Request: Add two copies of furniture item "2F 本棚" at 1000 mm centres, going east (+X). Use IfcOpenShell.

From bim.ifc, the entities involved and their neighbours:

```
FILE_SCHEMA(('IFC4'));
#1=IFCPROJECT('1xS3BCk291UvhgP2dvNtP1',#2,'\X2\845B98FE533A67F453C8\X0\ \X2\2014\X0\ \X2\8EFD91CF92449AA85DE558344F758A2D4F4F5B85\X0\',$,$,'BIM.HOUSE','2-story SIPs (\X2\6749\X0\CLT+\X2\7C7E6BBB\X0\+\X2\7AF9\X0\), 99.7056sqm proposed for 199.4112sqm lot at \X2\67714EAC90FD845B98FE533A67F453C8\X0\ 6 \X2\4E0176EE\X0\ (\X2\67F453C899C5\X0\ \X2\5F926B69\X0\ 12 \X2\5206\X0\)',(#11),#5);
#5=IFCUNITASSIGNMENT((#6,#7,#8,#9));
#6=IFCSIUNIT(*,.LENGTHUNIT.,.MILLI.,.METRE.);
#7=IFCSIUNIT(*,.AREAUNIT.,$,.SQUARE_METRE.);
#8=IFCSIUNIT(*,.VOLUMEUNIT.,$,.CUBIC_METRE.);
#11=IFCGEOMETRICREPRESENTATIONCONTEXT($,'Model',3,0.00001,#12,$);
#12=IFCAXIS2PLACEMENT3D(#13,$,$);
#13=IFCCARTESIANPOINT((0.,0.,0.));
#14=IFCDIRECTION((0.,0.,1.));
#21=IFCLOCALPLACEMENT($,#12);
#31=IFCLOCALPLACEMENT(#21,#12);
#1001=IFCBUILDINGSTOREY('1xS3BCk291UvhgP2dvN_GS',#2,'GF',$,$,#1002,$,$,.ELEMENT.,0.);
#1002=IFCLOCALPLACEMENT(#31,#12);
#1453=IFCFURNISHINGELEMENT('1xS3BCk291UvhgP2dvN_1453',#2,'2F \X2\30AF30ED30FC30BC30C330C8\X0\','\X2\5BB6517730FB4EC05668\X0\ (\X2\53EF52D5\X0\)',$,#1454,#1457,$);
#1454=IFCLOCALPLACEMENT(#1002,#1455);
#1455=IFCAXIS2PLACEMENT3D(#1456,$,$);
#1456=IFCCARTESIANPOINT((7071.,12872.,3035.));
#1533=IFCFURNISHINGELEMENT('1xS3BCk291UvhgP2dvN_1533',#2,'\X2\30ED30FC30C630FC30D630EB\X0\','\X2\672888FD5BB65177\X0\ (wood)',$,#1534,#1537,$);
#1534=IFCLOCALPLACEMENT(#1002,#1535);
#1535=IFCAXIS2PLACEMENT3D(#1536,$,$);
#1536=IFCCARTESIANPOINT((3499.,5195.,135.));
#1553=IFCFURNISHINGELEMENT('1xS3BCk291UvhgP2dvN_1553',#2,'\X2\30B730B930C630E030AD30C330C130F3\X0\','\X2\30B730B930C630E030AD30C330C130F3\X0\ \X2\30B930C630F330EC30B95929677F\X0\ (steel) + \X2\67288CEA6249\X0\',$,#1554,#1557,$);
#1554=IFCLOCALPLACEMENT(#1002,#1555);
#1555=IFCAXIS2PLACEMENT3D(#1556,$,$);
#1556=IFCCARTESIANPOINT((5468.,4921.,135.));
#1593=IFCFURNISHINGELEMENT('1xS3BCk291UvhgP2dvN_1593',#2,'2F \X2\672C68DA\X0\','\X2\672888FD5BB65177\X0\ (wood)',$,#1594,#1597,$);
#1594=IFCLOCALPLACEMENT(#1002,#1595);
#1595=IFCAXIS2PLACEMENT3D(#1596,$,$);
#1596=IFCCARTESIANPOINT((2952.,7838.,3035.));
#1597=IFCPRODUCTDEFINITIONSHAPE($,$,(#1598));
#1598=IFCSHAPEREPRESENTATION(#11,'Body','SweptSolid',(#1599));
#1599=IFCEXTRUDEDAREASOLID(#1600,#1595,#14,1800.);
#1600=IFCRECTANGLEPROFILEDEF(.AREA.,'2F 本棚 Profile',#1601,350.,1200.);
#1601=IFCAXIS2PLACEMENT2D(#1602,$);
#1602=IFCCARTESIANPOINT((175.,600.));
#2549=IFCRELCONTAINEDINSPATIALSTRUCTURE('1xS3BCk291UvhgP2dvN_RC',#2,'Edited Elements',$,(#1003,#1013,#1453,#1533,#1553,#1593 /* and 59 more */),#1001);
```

```python
import numpy as np
import ifcopenshell
import ifcopenshell.api.geometry
import ifcopenshell.api.root
import ifcopenshell.util.element
import ifcopenshell.util.placement
import ifcopenshell.util.unit

model = ifcopenshell.open("bim.ifc")
unit_scale = ifcopenshell.util.unit.calculate_unit_scale(model)


def reuse_history(source, copy):
    """copy_class also copies each property set's owner history, people and application; keep the originals."""
    for rel in copy.IsDefinedBy:
        if rel.is_a("IfcRelDefinesByProperties") and (history := rel.RelatingPropertyDefinition.OwnerHistory):
            rel.RelatingPropertyDefinition.OwnerHistory = source.OwnerHistory
            ifcopenshell.util.element.remove_deep2(model, history)


source = model.by_guid("1xS3BCk291UvhgP2dvN_1593")
base = ifcopenshell.util.placement.get_local_placement(source.ObjectPlacement)
step = np.array([1.0, 0.0, 0.0]) * 1 / unit_scale

for i in range(1, 3):
    copy = ifcopenshell.api.root.copy_class(model, product=source)
    copy.Representation = ifcopenshell.util.element.copy_deep(
        model, source.Representation, exclude=["IfcGeometricRepresentationContext", "IfcRepresentationMap"]
    )
    reuse_history(source, copy)
    matrix = base.copy()
    matrix[:3, 3] += i * step
    print("added at", matrix[:3, 3].round(3) + 0.0)
    ifcopenshell.api.geometry.edit_object_placement(model, product=copy, matrix=matrix, is_si=False)

model.write("bim_v2.ifc")
```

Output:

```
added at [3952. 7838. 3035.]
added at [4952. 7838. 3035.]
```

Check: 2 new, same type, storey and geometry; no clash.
